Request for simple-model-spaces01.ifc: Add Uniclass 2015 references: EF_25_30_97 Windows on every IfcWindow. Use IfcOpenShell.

First a look at what the model holds.

```python
import ifcopenshell

model = ifcopenshell.open("simple-model-spaces01.ifc")
print(model.schema)
print("classifications:", [c.Name for c in model.by_type("IfcClassification")])
for ifc_class in ("IfcDoor", "IfcRoof", "IfcStair", "IfcWall", "IfcWindow"):
    print(ifc_class, len(model.by_type(ifc_class)))
```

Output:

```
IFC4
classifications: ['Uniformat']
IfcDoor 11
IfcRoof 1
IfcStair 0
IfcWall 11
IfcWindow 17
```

```python
import ifcopenshell
import ifcopenshell.api.classification

model = ifcopenshell.open("simple-model-spaces01.ifc")

system = ifcopenshell.api.classification.add_classification(model, classification="Uniclass 2015")

codes = {
    "IfcWindow": ("EF_25_30_97", "Windows"),
}
for ifc_class, (code, name) in codes.items():
    products = model.by_type(ifc_class)
    ifcopenshell.api.classification.add_reference(
        model, products=products, classification=system, identification=code, name=name
    )
    print(code, len(products))

model.write("simple-model-spaces01_rev.ifc")
```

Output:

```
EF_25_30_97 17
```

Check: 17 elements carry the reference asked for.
